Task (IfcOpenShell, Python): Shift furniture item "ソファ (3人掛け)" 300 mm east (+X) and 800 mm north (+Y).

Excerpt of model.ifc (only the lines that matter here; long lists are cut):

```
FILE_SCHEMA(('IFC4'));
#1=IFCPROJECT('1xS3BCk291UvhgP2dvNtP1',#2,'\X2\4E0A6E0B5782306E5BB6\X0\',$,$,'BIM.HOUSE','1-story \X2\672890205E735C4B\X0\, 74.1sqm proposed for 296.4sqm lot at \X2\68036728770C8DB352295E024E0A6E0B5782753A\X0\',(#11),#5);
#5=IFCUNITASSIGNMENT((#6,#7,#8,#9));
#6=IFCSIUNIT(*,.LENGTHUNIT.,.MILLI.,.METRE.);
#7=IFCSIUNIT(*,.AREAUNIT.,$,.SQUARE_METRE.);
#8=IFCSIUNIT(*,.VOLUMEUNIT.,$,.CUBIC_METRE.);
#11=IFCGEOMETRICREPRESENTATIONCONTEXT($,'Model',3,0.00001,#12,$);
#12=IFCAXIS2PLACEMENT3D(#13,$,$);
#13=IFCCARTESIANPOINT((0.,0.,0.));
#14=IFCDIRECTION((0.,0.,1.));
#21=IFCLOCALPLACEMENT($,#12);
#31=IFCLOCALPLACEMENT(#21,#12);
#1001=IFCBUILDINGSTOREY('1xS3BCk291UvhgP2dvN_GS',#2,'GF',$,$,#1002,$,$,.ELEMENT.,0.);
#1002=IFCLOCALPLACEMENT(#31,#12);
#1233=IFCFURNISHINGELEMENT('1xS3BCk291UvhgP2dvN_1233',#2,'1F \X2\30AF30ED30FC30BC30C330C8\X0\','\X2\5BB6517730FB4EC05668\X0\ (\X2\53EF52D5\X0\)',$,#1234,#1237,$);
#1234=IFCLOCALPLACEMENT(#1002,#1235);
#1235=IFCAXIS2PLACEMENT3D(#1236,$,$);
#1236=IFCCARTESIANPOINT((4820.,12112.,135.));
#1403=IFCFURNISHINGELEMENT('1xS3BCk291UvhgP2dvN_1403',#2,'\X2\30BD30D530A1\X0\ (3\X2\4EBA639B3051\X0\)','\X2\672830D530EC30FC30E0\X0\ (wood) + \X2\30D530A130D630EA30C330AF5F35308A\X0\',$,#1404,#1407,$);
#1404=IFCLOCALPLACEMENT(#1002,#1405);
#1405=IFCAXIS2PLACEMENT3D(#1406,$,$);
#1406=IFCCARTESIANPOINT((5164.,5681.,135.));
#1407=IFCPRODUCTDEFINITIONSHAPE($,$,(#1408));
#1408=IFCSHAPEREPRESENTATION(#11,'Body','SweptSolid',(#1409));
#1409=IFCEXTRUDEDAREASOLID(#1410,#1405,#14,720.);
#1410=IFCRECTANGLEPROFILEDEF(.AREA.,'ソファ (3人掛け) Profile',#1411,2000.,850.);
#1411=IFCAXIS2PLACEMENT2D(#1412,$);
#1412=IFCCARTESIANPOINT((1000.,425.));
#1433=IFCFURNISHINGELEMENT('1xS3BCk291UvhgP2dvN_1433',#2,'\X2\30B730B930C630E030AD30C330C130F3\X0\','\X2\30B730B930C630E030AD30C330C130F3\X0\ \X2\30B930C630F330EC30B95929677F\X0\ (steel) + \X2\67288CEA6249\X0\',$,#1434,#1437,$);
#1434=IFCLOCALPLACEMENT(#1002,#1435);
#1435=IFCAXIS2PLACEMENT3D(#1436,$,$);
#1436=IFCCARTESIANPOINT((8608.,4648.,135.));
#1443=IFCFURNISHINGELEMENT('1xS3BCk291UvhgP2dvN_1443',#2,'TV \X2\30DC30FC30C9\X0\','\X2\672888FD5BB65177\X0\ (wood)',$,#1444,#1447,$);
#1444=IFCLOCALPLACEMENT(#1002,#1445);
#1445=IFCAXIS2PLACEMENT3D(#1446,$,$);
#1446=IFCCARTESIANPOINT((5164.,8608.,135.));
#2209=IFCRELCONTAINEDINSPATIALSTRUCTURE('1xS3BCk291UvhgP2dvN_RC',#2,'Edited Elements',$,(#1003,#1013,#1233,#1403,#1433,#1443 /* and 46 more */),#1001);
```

```python
import ifcopenshell
import ifcopenshell.api.geometry
import ifcopenshell.util.placement
import ifcopenshell.util.unit

model = ifcopenshell.open("model.ifc")
unit_scale = ifcopenshell.util.unit.calculate_unit_scale(model)

item = model.by_guid("1xS3BCk291UvhgP2dvN_1403")
matrix = ifcopenshell.util.placement.get_local_placement(item.ObjectPlacement)
matrix[0, 3] += 0.3 / unit_scale
matrix[1, 3] += 0.8 / unit_scale
ifcopenshell.api.geometry.edit_object_placement(model, product=item, matrix=matrix, is_si=False)

print(ifcopenshell.util.placement.get_local_placement(item.ObjectPlacement).round(3) + 0.0)

model.write("model_v2.ifc")
```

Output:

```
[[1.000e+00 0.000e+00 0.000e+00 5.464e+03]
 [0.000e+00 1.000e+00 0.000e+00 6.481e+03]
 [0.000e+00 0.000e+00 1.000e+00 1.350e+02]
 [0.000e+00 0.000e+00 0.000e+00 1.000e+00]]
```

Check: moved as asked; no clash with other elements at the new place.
